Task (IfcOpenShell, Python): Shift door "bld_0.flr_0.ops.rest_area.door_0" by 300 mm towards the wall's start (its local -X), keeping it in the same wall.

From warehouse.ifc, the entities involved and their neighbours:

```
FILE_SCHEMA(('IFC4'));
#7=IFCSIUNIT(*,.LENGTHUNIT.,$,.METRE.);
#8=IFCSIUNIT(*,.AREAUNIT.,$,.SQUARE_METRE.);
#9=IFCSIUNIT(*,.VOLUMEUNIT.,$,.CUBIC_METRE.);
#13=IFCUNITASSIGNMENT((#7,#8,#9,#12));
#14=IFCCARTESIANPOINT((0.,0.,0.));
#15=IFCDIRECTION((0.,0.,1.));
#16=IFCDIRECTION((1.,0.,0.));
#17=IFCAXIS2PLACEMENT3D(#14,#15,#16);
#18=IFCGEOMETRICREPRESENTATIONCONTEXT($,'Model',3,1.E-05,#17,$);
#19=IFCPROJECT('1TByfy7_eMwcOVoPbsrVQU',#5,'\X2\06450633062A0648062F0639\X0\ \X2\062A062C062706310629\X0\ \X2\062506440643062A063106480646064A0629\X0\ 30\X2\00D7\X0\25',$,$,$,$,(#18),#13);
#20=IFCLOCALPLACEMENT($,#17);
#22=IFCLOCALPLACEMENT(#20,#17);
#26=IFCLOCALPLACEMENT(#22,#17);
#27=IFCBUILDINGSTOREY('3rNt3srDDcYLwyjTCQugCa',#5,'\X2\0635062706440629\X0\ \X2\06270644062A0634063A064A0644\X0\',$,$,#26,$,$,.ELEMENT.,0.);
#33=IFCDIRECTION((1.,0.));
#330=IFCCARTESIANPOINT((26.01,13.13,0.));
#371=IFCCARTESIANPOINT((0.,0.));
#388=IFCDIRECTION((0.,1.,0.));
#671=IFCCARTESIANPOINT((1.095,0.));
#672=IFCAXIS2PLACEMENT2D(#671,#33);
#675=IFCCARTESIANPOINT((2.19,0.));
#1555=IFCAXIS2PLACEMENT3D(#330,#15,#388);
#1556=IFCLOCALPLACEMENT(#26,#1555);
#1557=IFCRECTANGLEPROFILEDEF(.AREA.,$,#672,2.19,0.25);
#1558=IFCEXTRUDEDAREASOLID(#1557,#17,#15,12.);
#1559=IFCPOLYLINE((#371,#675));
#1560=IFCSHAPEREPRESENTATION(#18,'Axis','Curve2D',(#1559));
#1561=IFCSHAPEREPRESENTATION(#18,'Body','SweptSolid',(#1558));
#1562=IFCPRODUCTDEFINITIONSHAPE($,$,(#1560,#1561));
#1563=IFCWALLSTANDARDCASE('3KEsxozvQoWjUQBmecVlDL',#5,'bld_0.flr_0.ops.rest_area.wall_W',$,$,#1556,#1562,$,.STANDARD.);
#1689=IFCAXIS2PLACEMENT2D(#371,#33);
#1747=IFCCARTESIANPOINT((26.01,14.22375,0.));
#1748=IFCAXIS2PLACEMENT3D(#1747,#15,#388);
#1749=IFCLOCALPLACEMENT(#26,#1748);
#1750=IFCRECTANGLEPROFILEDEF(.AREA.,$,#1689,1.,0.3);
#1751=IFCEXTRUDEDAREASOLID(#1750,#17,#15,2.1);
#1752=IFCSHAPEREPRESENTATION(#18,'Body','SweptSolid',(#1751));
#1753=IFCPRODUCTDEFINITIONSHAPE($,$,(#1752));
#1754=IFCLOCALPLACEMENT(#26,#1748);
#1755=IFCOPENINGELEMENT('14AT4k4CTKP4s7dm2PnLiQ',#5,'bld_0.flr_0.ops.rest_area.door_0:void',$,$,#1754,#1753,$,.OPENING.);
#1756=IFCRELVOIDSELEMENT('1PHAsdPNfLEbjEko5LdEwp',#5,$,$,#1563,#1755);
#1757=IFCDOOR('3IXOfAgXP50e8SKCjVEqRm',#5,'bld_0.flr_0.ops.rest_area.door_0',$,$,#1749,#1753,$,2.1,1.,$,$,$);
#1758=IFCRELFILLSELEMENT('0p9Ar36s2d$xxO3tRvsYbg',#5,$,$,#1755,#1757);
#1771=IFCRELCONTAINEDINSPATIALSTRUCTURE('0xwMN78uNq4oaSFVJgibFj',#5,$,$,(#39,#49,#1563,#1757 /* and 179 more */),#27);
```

```python
import ifcopenshell
import ifcopenshell.api.geometry
import ifcopenshell.util.placement
import ifcopenshell.util.unit

model = ifcopenshell.open("warehouse.ifc")
unit_scale = ifcopenshell.util.unit.calculate_unit_scale(model)

door = model.by_id(1757)
opening = door.FillsVoids[0].RelatingOpeningElement
wall = opening.VoidsElements[0].RelatingBuildingElement

wall_matrix = ifcopenshell.util.placement.get_local_placement(wall.ObjectPlacement)
shift = wall_matrix[:3, 0] * -0.3 / unit_scale
before = ifcopenshell.util.placement.get_local_placement(door.ObjectPlacement)[:3, 3].copy()

# The door is not placed relative to its opening, so move both.
for product in (opening, door):
    matrix = ifcopenshell.util.placement.get_local_placement(product.ObjectPlacement)
    matrix[:3, 3] += shift
    ifcopenshell.api.geometry.edit_object_placement(model, product=product, matrix=matrix, is_si=False)

after = ifcopenshell.util.placement.get_local_placement(door.ObjectPlacement)[:3, 3]
print("door moved by", (after - before).round(3) + 0.0)

model.write("warehouse_edited.ifc")
```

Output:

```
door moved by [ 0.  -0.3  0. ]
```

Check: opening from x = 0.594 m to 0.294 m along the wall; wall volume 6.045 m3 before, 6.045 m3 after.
